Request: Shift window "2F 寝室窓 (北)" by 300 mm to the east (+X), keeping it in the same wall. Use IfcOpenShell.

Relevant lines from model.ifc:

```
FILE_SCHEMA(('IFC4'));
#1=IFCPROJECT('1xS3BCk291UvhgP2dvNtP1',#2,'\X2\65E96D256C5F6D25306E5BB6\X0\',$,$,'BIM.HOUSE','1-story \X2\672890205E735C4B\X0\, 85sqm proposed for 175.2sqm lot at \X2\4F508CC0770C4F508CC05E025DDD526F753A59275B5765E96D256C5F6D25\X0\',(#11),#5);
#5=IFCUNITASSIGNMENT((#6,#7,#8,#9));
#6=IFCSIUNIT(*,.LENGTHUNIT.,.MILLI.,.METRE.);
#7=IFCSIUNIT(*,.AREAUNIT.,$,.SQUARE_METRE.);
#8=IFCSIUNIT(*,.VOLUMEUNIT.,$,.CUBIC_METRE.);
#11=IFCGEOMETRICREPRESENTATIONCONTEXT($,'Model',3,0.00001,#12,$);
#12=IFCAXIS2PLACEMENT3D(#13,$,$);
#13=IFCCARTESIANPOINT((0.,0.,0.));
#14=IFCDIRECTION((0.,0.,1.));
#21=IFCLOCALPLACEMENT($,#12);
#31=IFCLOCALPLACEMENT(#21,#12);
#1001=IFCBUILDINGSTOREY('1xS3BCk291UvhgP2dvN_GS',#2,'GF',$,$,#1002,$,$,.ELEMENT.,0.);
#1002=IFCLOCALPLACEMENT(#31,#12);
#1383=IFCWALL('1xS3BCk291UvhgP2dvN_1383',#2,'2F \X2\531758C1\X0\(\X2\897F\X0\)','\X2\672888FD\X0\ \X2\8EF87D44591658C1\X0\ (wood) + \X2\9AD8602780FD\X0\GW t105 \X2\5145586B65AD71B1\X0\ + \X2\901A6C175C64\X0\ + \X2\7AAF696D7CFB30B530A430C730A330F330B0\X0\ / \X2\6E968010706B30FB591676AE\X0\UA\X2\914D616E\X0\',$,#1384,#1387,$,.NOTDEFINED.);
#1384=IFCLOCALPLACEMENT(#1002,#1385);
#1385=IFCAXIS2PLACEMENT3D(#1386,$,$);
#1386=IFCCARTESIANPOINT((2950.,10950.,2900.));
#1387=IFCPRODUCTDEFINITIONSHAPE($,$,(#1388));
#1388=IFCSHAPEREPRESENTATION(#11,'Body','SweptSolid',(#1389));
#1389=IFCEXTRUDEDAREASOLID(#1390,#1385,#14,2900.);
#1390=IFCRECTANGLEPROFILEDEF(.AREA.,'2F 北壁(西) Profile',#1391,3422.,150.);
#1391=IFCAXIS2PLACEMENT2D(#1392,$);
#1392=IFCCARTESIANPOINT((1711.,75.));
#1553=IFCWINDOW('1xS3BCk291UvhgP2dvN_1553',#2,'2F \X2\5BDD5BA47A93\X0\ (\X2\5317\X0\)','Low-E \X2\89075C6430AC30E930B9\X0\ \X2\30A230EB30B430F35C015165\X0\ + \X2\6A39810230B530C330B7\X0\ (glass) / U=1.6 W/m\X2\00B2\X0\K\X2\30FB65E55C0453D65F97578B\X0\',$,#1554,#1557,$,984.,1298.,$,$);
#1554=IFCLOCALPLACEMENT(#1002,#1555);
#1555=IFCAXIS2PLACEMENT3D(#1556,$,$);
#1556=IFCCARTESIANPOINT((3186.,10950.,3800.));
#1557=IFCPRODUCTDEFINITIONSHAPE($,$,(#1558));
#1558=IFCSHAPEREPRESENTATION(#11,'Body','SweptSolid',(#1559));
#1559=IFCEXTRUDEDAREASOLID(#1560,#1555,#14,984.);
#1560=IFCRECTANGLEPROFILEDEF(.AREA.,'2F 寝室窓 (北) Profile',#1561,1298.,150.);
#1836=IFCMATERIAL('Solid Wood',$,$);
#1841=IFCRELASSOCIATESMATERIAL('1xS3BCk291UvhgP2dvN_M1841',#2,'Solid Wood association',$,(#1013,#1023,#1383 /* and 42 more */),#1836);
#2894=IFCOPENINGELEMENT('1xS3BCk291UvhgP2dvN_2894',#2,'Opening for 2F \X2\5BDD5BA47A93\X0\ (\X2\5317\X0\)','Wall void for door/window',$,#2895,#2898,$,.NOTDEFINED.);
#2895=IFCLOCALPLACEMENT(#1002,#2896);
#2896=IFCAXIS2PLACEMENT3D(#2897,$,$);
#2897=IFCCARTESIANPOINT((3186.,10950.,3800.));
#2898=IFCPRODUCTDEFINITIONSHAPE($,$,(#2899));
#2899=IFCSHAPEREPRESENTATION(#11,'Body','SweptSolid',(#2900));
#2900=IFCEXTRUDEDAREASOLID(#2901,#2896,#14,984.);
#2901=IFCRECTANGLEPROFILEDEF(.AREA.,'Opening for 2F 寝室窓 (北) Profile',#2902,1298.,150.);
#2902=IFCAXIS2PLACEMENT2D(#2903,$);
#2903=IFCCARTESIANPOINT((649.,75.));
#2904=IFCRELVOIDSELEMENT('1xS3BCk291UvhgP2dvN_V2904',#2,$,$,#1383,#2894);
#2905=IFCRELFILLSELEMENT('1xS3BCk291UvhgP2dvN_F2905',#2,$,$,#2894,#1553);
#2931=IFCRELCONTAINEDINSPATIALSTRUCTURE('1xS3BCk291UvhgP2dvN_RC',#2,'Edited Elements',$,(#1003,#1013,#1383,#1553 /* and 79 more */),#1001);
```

```python
import ifcopenshell
import ifcopenshell.api.geometry
import ifcopenshell.util.placement
import ifcopenshell.util.unit

model = ifcopenshell.open("model.ifc")
unit_scale = ifcopenshell.util.unit.calculate_unit_scale(model)

window = model.by_guid("1xS3BCk291UvhgP2dvN_1553")
opening = window.FillsVoids[0].RelatingOpeningElement
wall = opening.VoidsElements[0].RelatingBuildingElement

wall_matrix = ifcopenshell.util.placement.get_local_placement(wall.ObjectPlacement)
shift = wall_matrix[:3, 0] * 0.3 / unit_scale
before = ifcopenshell.util.placement.get_local_placement(window.ObjectPlacement)[:3, 3].copy()

# The window is not placed relative to its opening, so move both.
for product in (opening, window):
    matrix = ifcopenshell.util.placement.get_local_placement(product.ObjectPlacement)
    matrix[:3, 3] += shift
    ifcopenshell.api.geometry.edit_object_placement(model, product=product, matrix=matrix, is_si=False)

after = ifcopenshell.util.placement.get_local_placement(window.ObjectPlacement)[:3, 3]
print("window moved by", (after - before).round(3) + 0.0)

model.write("model_updated.ifc")
```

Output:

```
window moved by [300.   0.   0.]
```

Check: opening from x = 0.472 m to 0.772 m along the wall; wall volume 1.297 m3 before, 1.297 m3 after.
